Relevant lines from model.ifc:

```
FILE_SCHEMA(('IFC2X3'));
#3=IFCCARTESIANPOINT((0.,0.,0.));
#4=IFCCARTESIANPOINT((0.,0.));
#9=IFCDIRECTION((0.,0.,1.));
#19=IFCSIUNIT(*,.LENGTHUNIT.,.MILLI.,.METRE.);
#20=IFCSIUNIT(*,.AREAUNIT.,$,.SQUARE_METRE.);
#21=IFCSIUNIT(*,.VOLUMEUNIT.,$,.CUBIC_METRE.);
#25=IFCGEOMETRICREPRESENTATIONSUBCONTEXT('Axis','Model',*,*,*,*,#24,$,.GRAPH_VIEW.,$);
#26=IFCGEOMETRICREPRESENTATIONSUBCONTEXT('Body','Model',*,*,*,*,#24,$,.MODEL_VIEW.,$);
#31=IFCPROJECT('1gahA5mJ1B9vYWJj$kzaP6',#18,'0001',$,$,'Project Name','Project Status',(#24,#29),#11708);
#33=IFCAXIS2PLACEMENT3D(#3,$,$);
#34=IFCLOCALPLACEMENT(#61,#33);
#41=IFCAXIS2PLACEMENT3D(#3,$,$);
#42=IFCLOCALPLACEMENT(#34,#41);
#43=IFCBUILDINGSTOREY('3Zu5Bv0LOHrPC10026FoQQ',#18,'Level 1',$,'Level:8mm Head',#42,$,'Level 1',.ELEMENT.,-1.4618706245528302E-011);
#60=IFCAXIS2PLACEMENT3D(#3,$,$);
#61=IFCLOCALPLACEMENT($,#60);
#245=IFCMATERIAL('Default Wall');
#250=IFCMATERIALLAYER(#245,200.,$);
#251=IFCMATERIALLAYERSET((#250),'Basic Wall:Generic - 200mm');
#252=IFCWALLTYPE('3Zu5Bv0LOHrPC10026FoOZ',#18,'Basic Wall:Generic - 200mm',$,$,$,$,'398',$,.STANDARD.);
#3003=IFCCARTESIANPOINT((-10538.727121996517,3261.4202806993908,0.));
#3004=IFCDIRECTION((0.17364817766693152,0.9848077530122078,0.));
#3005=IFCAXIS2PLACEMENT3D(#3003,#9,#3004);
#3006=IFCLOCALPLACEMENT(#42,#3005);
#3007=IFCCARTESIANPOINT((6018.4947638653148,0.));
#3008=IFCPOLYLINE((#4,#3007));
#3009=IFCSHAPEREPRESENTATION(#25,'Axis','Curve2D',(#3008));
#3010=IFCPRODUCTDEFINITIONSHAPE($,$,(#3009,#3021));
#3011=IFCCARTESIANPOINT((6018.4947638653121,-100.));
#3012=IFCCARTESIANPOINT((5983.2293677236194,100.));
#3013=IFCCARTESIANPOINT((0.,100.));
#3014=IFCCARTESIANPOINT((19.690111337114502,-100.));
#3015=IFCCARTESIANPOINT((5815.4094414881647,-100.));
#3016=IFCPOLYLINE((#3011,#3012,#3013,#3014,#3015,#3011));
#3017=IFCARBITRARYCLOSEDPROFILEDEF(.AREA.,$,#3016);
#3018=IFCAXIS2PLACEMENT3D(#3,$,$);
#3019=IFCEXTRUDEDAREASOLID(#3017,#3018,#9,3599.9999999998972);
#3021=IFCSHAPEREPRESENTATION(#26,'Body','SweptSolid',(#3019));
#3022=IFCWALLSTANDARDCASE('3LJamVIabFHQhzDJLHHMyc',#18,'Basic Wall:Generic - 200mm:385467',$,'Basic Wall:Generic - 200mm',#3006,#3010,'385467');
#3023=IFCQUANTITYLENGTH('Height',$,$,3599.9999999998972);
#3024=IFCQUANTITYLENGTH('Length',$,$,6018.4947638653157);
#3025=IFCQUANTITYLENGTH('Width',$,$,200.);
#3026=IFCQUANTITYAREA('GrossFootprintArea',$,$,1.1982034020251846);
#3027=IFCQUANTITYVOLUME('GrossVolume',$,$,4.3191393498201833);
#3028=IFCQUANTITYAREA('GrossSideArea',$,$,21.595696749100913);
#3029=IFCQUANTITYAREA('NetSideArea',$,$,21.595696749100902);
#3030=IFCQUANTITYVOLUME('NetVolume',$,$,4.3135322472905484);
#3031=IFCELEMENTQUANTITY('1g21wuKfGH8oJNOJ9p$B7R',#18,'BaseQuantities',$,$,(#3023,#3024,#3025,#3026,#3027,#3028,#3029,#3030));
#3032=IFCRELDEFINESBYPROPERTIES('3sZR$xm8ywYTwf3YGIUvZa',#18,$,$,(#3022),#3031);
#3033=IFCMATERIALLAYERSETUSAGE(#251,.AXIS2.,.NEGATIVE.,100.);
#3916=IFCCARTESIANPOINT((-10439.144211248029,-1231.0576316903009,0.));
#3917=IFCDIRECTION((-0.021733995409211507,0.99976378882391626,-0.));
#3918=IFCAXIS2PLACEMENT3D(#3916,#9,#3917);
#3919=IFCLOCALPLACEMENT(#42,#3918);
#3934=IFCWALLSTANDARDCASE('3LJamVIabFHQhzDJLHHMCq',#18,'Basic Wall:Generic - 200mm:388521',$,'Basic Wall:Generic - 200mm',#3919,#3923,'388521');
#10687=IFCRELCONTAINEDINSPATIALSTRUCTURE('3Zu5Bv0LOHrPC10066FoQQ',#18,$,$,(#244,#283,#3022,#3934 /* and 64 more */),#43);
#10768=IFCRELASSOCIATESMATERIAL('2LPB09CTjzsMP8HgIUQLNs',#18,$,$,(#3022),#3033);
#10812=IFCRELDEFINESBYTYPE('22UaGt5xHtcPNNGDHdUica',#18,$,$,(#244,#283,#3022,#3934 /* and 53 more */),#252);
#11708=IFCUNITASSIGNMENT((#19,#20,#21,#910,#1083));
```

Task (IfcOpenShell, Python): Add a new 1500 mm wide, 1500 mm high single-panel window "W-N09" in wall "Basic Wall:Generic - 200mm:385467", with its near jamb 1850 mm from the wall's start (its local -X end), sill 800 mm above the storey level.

```python
import numpy as np
import ifcopenshell
import ifcopenshell.api.feature
import ifcopenshell.api.geometry
import ifcopenshell.api.pset
import ifcopenshell.api.root
import ifcopenshell.api.spatial
import ifcopenshell.api.type
import ifcopenshell.geom
import ifcopenshell.util.element
import ifcopenshell.util.placement
import ifcopenshell.util.representation
import ifcopenshell.util.shape
import ifcopenshell.util.unit

model = ifcopenshell.open("model.ifc")
unit_scale = ifcopenshell.util.unit.calculate_unit_scale(model)
area_scale = ifcopenshell.util.unit.calculate_unit_scale(model, "AREAUNIT")
volume_scale = ifcopenshell.util.unit.calculate_unit_scale(model, "VOLUMEUNIT")
settings = ifcopenshell.geom.settings()


def volume(element):
    """Net volume in cubic metres, openings subtracted."""
    shape = ifcopenshell.geom.create_shape(settings, element)
    return ifcopenshell.util.shape.get_volume(shape.geometry)


wall = model.by_guid("3LJamVIabFHQhzDJLHHMyc")
storey = ifcopenshell.util.element.get_container(wall, ifc_class="IfcBuildingStorey")
context = ifcopenshell.util.representation.get_context(model, "Model", "Body", "MODEL_VIEW")
before = volume(wall)

width, height, from_end, sill = 1.5, 1.5, 1.85, 0.8  # metres

# The wall runs along its own X axis, and the end named is its -X end.
wall_shape = ifcopenshell.geom.create_shape(settings, wall)
x, y, z = ifcopenshell.util.shape.get_vertices(wall_shape.geometry).T
start = x.min() + from_end
face, thickness = float(y.min()), float(y.max() - y.min())
wall_matrix = ifcopenshell.util.placement.get_local_placement(wall.ObjectPlacement)
level = ifcopenshell.util.placement.get_local_placement(storey.ObjectPlacement)[2, 3]


def in_wall(x, y):
    """Placement at x, y metres in the wall's axes, at sill height."""
    matrix = wall_matrix.copy()
    matrix[:, 3] = wall_matrix @ np.array([x / unit_scale, y / unit_scale, 0.0, 1.0])
    matrix[2, 3] = level + sill / unit_scale
    return matrix


# Opening: a box that overshoots both wall faces by 50 mm.
opening = ifcopenshell.api.root.create_entity(model, ifc_class="IfcOpeningElement")
box = ifcopenshell.api.geometry.add_wall_representation(
    model, context=context, length=width, height=height, thickness=thickness + 0.1
)
ifcopenshell.api.geometry.assign_representation(model, product=opening, representation=box)
ifcopenshell.api.geometry.edit_object_placement(model, product=opening, matrix=in_wall(start, face - 0.05), is_si=False)
ifcopenshell.api.feature.add_feature(model, feature=opening, element=wall)

window = ifcopenshell.api.root.create_entity(model, ifc_class="IfcWindow", name="W-N09")
window.OverallWidth, window.OverallHeight = width / unit_scale, height / unit_scale
body = ifcopenshell.api.geometry.add_window_representation(
    model,
    context=context,
    overall_width=window.OverallWidth,
    overall_height=window.OverallHeight,
    partition_type="SINGLE_PANEL",
)
ifcopenshell.api.geometry.assign_representation(model, product=window, representation=body)
ifcopenshell.api.spatial.assign_container(model, products=[window], relating_structure=storey)
fills = ifcopenshell.api.feature.add_filling(model, opening=opening, element=window)
fills.OwnerHistory = window.OwnerHistory  # required in IFC2X3

# IFC2X3 keeps the operation on the window style.
style = ifcopenshell.api.root.create_entity(model, ifc_class="IfcWindowStyle", name="W-N09")
style.OperationType, style.ConstructionType = "SINGLE_PANEL", "NOTDEFINED"
style.ParameterTakesPrecedence = style.Sizeable = False
ifcopenshell.api.type.assign_type(model, related_objects=[window], relating_type=style)

# Centre the window in the wall's thickness.
ifcopenshell.api.geometry.edit_object_placement(model, product=window, matrix=in_wall(start, face), is_si=False)
window_shape = ifcopenshell.geom.create_shape(settings, window)
depth = ifcopenshell.util.shape.get_vertices(window_shape.geometry)[:, 1]
offset = face + thickness / 2 - (depth.min() + depth.max()) / 2
ifcopenshell.api.geometry.edit_object_placement(model, product=window, matrix=in_wall(start, offset), is_si=False)

after = volume(wall)

# Update the wall's stored quantities.
qto = model.by_id(ifcopenshell.util.element.get_pset(wall, "BaseQuantities", should_inherit=False)["id"])
ifcopenshell.api.pset.edit_qto(model, qto=qto, properties={
    "NetSideArea": after / thickness / area_scale,
    "NetVolume": after / volume_scale,
})

print(f"wall volume {before:.3f} -> {after:.3f} m3")

model.write("model_edited.ifc")
```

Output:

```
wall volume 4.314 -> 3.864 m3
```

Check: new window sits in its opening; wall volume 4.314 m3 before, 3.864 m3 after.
